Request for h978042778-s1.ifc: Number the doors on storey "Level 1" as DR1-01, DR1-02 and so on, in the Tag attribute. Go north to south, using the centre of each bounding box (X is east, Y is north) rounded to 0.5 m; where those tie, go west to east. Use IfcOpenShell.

First a look at what the model holds.

```python
import ifcopenshell
import ifcopenshell.util.element
import ifcopenshell.util.placement

model = ifcopenshell.open("h978042778-s1.ifc")
print(model.schema)
storey = next(s for s in model.by_type("IfcBuildingStorey") if s.Name == "Level 1")
doors = [e for e in ifcopenshell.util.element.get_decomposition(storey) if e.is_a("IfcDoor")]
for e in sorted(doors, key=lambda e: e.id()):
    origin = ifcopenshell.util.placement.get_local_placement(e.ObjectPlacement)[:3, 3]
    print(e.id(), e.Tag, e.Name, origin.round(2) + 0.0, sep=" | ")
```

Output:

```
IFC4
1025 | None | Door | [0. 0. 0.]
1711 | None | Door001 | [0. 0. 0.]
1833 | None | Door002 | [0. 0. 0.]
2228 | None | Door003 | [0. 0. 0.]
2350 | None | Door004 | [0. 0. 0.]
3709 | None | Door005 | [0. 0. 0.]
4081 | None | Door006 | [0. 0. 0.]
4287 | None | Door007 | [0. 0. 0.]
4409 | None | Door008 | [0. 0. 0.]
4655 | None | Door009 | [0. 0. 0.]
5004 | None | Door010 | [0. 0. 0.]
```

```python
import ifcopenshell
import ifcopenshell.geom
import ifcopenshell.util.element
import ifcopenshell.util.shape

model = ifcopenshell.open("h978042778-s1.ifc")
settings = ifcopenshell.geom.settings()
settings.set("use-world-coords", True)


def centre(element):
    shape = ifcopenshell.geom.create_shape(settings, element)
    return ifcopenshell.util.shape.get_bbox_centroid(shape.geometry)


storey = next(s for s in model.by_type("IfcBuildingStorey") if s.Name == "Level 1")
doors = [e for e in ifcopenshell.util.element.get_decomposition(storey) if e.is_a("IfcDoor")]

# Insertion points can sit at a corner or the storey origin, so sort by the geometry (in metres).
centres = {e: centre(e) for e in doors}
doors.sort(key=lambda e: (-round(centres[e][1] / 0.5), centres[e][0]))

for i, e in enumerate(doors, start=1):
    number = f"DR1-{i:02d}"
    e.Tag = number
    print(e.id(), number)

model.write("h978042778-s1_v2.ifc")
```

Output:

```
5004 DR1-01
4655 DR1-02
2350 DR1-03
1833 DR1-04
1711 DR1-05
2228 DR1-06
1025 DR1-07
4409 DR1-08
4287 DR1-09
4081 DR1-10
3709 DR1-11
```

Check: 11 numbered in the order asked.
